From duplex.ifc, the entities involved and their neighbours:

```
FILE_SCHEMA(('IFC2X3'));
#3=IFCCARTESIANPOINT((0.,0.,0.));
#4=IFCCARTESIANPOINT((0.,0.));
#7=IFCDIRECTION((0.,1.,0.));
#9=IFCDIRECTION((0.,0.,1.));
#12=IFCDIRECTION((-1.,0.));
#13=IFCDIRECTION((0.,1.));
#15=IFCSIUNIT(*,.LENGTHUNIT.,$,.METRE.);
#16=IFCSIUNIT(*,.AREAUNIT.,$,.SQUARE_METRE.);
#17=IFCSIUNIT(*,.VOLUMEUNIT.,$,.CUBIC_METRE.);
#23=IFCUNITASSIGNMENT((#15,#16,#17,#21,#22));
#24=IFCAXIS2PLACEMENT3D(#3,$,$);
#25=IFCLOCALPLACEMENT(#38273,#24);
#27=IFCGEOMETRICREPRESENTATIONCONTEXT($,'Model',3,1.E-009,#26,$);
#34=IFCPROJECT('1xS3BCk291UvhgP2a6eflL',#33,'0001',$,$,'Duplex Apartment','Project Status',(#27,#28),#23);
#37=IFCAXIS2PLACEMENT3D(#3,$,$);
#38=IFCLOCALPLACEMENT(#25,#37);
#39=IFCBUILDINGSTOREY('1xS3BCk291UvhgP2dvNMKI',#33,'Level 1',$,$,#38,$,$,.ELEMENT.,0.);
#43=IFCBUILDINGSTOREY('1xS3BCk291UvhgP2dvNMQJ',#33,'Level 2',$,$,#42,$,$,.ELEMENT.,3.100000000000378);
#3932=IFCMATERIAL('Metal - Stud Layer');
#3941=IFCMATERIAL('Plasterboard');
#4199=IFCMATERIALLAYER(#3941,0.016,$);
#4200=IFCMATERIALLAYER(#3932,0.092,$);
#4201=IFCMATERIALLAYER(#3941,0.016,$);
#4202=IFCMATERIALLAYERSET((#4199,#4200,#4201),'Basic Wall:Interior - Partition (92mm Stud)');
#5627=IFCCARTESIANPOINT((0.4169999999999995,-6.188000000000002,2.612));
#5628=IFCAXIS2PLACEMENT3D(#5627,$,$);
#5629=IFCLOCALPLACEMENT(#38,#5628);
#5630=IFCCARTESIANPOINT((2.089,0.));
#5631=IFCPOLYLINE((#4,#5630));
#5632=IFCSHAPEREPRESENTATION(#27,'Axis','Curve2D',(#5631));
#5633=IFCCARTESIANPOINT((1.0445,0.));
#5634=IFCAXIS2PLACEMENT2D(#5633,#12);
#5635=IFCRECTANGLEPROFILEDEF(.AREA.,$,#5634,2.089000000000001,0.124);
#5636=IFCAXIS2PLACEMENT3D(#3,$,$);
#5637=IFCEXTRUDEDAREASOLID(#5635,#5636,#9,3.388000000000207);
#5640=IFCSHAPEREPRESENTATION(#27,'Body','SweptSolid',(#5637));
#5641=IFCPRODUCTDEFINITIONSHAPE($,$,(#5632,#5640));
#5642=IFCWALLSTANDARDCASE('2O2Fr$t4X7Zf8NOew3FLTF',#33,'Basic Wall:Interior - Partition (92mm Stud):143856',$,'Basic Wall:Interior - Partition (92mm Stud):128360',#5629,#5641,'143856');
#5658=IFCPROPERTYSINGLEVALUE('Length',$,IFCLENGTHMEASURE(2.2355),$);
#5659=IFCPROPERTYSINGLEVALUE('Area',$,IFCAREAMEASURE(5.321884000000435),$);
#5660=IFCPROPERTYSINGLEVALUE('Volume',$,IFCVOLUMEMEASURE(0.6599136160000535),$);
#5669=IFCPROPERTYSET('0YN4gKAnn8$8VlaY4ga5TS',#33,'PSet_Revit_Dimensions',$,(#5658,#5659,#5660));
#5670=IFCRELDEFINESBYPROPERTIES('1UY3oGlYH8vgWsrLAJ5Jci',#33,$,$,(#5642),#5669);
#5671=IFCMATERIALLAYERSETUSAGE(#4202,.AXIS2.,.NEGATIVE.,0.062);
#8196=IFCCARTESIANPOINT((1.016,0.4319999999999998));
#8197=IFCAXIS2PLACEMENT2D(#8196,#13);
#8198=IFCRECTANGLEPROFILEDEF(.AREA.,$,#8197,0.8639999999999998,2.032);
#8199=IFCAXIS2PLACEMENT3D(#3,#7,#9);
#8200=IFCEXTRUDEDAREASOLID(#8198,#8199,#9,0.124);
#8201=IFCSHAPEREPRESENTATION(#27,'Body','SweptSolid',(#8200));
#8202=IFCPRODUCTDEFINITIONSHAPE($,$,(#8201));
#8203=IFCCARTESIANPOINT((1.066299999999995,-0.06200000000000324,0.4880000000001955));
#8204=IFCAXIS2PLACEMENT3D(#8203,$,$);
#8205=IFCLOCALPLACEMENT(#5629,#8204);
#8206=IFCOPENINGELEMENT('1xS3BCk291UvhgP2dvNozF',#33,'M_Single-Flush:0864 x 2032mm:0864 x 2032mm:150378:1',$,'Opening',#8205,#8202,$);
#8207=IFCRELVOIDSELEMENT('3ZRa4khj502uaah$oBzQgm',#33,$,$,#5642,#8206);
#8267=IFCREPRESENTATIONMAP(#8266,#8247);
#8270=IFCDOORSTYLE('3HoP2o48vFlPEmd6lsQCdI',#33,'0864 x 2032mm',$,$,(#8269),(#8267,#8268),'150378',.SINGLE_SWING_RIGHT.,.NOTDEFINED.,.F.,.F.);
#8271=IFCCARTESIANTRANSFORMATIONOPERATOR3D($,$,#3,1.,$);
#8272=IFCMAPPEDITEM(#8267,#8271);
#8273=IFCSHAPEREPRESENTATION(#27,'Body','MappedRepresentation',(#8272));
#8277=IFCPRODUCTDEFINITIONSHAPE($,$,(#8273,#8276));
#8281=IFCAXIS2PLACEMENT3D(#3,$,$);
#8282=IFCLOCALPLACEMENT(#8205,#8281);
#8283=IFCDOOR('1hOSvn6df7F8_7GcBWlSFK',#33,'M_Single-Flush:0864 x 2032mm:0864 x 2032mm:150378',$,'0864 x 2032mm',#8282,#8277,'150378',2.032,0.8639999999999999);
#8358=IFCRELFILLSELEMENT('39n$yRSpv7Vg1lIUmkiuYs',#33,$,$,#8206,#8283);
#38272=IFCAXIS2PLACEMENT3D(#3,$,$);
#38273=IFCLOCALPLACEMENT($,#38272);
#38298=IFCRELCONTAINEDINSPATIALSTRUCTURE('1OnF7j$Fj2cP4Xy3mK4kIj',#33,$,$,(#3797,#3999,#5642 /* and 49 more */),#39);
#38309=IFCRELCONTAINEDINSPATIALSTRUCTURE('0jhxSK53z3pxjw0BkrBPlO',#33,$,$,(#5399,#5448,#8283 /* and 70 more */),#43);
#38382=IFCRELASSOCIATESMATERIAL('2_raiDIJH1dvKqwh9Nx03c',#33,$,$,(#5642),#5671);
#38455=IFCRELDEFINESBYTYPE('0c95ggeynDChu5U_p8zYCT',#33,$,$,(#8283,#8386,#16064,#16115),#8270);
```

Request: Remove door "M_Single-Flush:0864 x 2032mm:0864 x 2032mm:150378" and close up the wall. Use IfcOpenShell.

```python
import ifcopenshell
import ifcopenshell.api.feature
import ifcopenshell.api.pset
import ifcopenshell.api.root
import ifcopenshell.geom
import ifcopenshell.util.element
import ifcopenshell.util.shape
import ifcopenshell.util.unit

model = ifcopenshell.open("duplex.ifc")
area_scale = ifcopenshell.util.unit.calculate_unit_scale(model, "AREAUNIT")
volume_scale = ifcopenshell.util.unit.calculate_unit_scale(model, "VOLUMEUNIT")
settings = ifcopenshell.geom.settings()


def volume(element):
    """Net volume in cubic metres, openings subtracted."""
    shape = ifcopenshell.geom.create_shape(settings, element)
    return ifcopenshell.util.shape.get_volume(shape.geometry)


door = model.by_id(8283)
opening = door.FillsVoids[0].RelatingOpeningElement
wall = opening.VoidsElements[0].RelatingBuildingElement
before = volume(wall)

ifcopenshell.api.root.remove_product(model, product=door)
ifcopenshell.api.feature.remove_feature(model, feature=opening)

after = volume(wall)
thickness = 0.124  # wall thickness in metres

# Update the wall's stored quantities.
pset = model.by_id(ifcopenshell.util.element.get_pset(wall, "PSet_Revit_Dimensions", should_inherit=False)["id"])
ifcopenshell.api.pset.edit_pset(model, pset=pset, properties={
    "Area": model.create_entity("IfcAreaMeasure", after / thickness / area_scale),
    "Volume": model.create_entity("IfcVolumeMeasure", after / volume_scale),
})

print(f"wall volume {before:.3f} -> {after:.3f} m3")

model.write("duplex_v2.ifc")
```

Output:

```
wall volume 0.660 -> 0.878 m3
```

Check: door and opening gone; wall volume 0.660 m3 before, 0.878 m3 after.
